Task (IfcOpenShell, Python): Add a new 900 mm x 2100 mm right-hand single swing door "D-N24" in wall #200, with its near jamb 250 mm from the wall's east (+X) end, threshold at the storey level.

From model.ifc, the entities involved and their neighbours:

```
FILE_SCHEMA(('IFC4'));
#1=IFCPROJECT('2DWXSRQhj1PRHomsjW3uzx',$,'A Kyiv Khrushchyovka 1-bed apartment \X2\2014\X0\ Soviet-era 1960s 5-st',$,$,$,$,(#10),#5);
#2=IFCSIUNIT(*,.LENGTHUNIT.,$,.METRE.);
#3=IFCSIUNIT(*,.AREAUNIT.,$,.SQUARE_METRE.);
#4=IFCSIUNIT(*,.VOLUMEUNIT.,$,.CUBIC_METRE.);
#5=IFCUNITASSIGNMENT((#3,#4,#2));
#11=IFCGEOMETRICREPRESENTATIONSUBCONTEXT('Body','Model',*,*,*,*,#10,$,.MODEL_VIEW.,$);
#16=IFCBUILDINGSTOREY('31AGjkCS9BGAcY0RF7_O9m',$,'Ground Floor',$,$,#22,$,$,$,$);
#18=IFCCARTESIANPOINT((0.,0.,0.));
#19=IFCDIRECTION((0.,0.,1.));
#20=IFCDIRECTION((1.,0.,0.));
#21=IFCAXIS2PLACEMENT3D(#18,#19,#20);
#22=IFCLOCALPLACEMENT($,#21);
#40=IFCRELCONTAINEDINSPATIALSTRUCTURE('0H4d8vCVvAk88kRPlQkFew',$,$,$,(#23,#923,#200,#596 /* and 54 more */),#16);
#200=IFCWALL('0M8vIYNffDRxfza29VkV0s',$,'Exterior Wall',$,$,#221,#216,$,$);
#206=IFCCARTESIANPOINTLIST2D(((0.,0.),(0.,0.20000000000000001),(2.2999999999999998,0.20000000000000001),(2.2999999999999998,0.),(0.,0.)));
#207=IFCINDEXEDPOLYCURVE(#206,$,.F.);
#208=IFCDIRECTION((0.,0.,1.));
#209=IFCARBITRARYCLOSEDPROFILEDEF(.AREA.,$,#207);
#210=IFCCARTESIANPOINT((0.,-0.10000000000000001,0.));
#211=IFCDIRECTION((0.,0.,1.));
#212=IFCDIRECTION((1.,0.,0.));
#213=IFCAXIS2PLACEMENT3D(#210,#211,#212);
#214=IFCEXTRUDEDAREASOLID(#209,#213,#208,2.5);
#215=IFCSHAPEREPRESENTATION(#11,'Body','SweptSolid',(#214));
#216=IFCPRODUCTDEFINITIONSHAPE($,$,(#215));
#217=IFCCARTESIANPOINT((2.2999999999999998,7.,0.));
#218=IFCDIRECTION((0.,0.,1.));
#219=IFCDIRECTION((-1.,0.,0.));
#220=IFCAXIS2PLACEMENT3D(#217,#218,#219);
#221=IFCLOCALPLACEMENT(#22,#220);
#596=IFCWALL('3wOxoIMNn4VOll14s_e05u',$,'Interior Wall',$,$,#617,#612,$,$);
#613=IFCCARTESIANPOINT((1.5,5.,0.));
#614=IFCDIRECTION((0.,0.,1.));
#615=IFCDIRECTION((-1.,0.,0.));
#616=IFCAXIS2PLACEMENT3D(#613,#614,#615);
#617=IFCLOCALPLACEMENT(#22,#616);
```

```python
import numpy as np
import ifcopenshell
import ifcopenshell.api.feature
import ifcopenshell.api.geometry
import ifcopenshell.api.root
import ifcopenshell.api.spatial
import ifcopenshell.geom
import ifcopenshell.util.element
import ifcopenshell.util.placement
import ifcopenshell.util.representation
import ifcopenshell.util.shape
import ifcopenshell.util.unit

model = ifcopenshell.open("model.ifc")
unit_scale = ifcopenshell.util.unit.calculate_unit_scale(model)
settings = ifcopenshell.geom.settings()


def volume(element):
    """Net volume in cubic metres, openings subtracted."""
    shape = ifcopenshell.geom.create_shape(settings, element)
    return ifcopenshell.util.shape.get_volume(shape.geometry)


wall = model.by_guid("0M8vIYNffDRxfza29VkV0s")
storey = ifcopenshell.util.element.get_container(wall, ifc_class="IfcBuildingStorey")
context = ifcopenshell.util.representation.get_context(model, "Model", "Body", "MODEL_VIEW")
before = volume(wall)

width, height, from_end, sill = 0.9, 2.1, 0.25, 0.0  # metres

# The wall runs along its own X axis, and the end named is its -X end.
wall_shape = ifcopenshell.geom.create_shape(settings, wall)
x, y, z = ifcopenshell.util.shape.get_vertices(wall_shape.geometry).T
start = x.min() + from_end
face, thickness = float(y.min()), float(y.max() - y.min())
wall_matrix = ifcopenshell.util.placement.get_local_placement(wall.ObjectPlacement)
level = ifcopenshell.util.placement.get_local_placement(storey.ObjectPlacement)[2, 3]


def in_wall(x, y):
    """Placement at x, y metres in the wall's axes, at sill height."""
    matrix = wall_matrix.copy()
    matrix[:, 3] = wall_matrix @ np.array([x / unit_scale, y / unit_scale, 0.0, 1.0])
    matrix[2, 3] = level + sill / unit_scale
    return matrix


# Opening: a box that overshoots both wall faces by 50 mm.
opening = ifcopenshell.api.root.create_entity(model, ifc_class="IfcOpeningElement", predefined_type="OPENING")
box = ifcopenshell.api.geometry.add_wall_representation(
    model, context=context, length=width, height=height, thickness=thickness + 0.1
)
ifcopenshell.api.geometry.assign_representation(model, product=opening, representation=box)
ifcopenshell.api.geometry.edit_object_placement(model, product=opening, matrix=in_wall(start, face - 0.05), is_si=False)
ifcopenshell.api.feature.add_feature(model, feature=opening, element=wall)

door = ifcopenshell.api.root.create_entity(model, ifc_class="IfcDoor", name="D-N24", predefined_type="DOOR")
door.OverallWidth, door.OverallHeight = width / unit_scale, height / unit_scale
door.OperationType = "SINGLE_SWING_RIGHT"
body = ifcopenshell.api.geometry.add_door_representation(
    model,
    context=context,
    overall_width=door.OverallWidth,
    overall_height=door.OverallHeight,
    operation_type="SINGLE_SWING_RIGHT",
    lining_properties={"LiningDepth": thickness / unit_scale, "ThresholdDepth": thickness / unit_scale},
)
ifcopenshell.api.geometry.assign_representation(model, product=door, representation=body)
ifcopenshell.api.spatial.assign_container(model, products=[door], relating_structure=storey)
ifcopenshell.api.feature.add_filling(model, opening=opening, element=door)

# The lining spans the wall, so the door starts at the wall face.
ifcopenshell.api.geometry.edit_object_placement(model, product=door, matrix=in_wall(start, face), is_si=False)

after = volume(wall)

print(f"wall volume {before:.3f} -> {after:.3f} m3")

model.write("model_v2.ifc")
```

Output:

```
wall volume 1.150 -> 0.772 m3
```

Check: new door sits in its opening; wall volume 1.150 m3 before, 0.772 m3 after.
